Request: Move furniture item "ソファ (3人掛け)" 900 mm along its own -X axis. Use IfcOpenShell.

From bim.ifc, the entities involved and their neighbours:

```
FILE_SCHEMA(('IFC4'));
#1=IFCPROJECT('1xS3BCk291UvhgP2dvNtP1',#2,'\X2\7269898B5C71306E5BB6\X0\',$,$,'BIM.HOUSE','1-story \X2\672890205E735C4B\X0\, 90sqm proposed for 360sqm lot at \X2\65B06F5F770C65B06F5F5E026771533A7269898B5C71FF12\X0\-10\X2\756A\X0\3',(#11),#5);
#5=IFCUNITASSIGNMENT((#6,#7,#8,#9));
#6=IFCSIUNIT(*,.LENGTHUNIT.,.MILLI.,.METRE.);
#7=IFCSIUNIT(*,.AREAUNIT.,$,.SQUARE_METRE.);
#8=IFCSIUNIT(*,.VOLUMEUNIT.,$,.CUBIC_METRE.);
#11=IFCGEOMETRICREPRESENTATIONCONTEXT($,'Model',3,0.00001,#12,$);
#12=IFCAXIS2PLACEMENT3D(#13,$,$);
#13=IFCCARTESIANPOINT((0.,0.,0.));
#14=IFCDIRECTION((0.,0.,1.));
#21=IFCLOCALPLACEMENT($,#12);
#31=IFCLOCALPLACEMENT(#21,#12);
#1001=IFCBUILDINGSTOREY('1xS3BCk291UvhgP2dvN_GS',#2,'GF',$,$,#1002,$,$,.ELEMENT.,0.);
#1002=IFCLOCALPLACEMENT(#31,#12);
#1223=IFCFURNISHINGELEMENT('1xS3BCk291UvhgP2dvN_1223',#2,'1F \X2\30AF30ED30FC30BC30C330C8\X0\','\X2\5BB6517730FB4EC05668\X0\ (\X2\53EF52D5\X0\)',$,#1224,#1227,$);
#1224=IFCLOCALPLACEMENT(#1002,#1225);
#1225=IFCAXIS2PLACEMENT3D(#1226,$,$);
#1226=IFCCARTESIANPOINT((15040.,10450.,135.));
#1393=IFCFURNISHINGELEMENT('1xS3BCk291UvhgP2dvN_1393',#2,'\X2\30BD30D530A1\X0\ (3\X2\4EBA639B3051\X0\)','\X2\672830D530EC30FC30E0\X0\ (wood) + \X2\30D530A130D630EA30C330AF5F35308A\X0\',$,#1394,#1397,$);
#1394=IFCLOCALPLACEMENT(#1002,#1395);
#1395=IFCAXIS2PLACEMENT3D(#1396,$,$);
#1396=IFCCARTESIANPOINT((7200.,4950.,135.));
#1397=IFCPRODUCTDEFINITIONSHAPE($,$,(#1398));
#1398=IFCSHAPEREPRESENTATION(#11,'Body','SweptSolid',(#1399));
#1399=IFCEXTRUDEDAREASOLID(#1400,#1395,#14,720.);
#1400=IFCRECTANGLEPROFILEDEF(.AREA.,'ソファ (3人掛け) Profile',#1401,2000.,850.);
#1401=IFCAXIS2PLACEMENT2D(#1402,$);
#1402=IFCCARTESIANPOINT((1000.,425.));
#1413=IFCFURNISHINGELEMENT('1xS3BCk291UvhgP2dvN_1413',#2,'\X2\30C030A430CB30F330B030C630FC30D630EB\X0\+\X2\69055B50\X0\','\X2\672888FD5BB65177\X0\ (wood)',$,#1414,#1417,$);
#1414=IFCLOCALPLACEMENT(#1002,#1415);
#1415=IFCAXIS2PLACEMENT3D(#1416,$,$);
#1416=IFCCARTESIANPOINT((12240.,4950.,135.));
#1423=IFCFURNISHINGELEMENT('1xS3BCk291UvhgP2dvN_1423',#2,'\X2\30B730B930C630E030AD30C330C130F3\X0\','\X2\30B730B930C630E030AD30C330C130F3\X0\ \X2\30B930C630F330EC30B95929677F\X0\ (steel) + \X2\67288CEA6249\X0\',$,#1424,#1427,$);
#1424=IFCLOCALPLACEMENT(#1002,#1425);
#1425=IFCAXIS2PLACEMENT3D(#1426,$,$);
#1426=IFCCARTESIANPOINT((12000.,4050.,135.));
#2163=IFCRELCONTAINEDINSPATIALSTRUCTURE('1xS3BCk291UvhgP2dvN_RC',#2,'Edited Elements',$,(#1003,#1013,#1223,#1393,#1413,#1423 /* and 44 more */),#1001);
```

```python
import ifcopenshell
import ifcopenshell.api.geometry
import ifcopenshell.util.placement

model = ifcopenshell.open("bim.ifc")

item = model.by_id(1393)
matrix = ifcopenshell.util.placement.get_local_placement(item.ObjectPlacement)
matrix[:3, 3] -= matrix[:3, 0] * 900.0
ifcopenshell.api.geometry.edit_object_placement(model, product=item, matrix=matrix, is_si=False)

print(ifcopenshell.util.placement.get_local_placement(item.ObjectPlacement).round(3) + 0.0)

model.write("bim_edited.ifc")
```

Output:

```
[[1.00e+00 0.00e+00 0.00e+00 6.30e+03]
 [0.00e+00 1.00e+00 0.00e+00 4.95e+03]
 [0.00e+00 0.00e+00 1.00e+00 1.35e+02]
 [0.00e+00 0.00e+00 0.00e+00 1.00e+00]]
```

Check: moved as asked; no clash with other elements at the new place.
